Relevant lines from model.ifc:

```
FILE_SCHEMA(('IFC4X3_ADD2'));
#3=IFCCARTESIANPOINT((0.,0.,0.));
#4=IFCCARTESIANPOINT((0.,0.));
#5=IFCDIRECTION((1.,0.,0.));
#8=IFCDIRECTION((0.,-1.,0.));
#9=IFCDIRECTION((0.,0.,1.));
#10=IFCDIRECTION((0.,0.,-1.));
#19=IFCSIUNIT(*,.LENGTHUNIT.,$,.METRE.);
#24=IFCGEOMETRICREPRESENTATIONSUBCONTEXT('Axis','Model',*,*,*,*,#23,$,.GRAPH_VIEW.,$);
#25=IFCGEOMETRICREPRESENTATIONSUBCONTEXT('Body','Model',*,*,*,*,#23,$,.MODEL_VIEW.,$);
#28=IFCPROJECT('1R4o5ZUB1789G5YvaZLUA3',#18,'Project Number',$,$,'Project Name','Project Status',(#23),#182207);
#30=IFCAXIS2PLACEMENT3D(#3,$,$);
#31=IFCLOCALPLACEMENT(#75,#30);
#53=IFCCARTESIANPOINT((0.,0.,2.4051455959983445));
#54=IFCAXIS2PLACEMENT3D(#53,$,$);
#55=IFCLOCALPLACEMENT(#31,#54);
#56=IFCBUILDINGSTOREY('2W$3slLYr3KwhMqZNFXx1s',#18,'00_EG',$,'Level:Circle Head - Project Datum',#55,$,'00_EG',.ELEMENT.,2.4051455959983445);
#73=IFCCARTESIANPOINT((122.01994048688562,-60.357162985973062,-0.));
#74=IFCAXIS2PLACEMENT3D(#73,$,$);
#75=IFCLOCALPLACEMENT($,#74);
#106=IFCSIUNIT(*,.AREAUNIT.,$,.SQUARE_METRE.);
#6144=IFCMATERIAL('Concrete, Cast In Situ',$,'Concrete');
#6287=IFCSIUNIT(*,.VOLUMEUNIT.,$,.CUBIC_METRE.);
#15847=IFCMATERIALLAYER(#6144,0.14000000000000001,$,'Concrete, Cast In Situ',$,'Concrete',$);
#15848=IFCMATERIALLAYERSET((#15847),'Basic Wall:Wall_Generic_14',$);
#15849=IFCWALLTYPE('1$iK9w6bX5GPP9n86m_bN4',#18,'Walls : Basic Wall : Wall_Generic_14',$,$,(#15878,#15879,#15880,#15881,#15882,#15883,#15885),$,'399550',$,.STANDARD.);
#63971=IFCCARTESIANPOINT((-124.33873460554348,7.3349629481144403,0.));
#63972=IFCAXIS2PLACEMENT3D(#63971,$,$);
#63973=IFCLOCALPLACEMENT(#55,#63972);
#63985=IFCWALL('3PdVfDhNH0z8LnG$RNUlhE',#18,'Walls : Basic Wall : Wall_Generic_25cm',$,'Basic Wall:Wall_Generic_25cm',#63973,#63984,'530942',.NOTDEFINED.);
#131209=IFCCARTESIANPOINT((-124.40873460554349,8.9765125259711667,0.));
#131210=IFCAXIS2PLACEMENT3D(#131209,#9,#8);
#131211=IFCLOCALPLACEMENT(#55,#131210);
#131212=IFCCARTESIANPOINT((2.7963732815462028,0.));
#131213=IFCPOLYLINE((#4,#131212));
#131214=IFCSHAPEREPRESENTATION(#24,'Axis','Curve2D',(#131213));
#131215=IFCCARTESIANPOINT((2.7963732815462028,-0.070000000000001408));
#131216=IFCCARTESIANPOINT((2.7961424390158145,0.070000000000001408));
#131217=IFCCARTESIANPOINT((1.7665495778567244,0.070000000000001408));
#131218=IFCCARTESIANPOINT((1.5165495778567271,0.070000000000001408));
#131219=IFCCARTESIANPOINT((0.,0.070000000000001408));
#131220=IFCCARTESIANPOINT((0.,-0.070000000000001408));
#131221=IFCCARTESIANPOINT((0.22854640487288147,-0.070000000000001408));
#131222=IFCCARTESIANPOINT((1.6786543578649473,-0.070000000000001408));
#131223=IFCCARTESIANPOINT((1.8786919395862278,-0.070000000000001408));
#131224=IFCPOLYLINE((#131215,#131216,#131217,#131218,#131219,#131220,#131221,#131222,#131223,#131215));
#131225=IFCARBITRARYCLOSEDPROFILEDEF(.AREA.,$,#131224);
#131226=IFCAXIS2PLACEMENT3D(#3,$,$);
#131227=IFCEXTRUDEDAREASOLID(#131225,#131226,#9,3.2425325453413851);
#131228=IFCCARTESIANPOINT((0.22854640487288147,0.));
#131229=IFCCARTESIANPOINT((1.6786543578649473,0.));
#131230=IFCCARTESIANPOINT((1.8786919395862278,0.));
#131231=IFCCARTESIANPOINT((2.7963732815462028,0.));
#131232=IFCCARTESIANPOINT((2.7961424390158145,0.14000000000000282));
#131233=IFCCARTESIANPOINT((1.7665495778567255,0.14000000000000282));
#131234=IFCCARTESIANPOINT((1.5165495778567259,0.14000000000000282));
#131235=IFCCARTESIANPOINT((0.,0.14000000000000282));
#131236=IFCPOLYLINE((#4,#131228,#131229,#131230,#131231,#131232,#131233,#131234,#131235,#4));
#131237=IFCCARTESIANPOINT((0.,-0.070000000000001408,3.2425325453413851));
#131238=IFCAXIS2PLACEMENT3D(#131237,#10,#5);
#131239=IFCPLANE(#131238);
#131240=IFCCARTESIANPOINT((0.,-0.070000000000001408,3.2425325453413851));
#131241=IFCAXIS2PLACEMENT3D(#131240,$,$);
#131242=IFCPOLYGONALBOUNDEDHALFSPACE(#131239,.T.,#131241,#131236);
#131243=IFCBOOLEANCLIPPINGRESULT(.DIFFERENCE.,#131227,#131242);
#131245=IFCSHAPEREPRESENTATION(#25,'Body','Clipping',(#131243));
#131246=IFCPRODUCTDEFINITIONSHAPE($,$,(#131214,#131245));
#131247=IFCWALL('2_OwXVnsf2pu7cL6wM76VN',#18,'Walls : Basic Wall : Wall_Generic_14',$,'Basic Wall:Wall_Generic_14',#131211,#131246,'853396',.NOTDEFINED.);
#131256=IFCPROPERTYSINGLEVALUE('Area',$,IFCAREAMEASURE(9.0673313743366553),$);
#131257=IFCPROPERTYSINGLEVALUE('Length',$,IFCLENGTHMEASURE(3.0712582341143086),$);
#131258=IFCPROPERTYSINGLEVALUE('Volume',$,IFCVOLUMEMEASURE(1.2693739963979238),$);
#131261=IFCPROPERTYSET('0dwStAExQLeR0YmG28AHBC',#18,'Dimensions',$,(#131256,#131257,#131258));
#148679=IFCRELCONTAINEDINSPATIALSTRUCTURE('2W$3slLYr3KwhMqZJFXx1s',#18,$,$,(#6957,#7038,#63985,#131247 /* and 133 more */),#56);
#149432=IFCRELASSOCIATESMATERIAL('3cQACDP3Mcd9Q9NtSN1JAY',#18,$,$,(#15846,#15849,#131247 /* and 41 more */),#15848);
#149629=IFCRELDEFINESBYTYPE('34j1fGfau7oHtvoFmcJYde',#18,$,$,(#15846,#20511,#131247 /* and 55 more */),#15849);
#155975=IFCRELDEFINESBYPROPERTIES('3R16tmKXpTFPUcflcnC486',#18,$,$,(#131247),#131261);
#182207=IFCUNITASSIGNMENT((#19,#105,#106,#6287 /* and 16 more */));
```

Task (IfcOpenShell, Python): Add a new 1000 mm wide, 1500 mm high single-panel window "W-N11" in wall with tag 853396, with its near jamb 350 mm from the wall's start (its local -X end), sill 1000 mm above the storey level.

```python
import numpy as np
import ifcopenshell
import ifcopenshell.api.feature
import ifcopenshell.api.geometry
import ifcopenshell.api.pset
import ifcopenshell.api.root
import ifcopenshell.api.spatial
import ifcopenshell.geom
import ifcopenshell.util.element
import ifcopenshell.util.placement
import ifcopenshell.util.representation
import ifcopenshell.util.shape
import ifcopenshell.util.unit

model = ifcopenshell.open("model.ifc")
unit_scale = ifcopenshell.util.unit.calculate_unit_scale(model)
area_scale = ifcopenshell.util.unit.calculate_unit_scale(model, "AREAUNIT")
volume_scale = ifcopenshell.util.unit.calculate_unit_scale(model, "VOLUMEUNIT")
settings = ifcopenshell.geom.settings()


def volume(element):
    """Net volume in cubic metres, openings subtracted."""
    shape = ifcopenshell.geom.create_shape(settings, element)
    return ifcopenshell.util.shape.get_volume(shape.geometry)


wall = model.by_guid("2_OwXVnsf2pu7cL6wM76VN")
storey = ifcopenshell.util.element.get_container(wall, ifc_class="IfcBuildingStorey")
context = ifcopenshell.util.representation.get_context(model, "Model", "Body", "MODEL_VIEW")
before = volume(wall)

width, height, from_end, sill = 1, 1.5, 0.35, 1  # metres

# The wall runs along its own X axis, and the end named is its -X end.
wall_shape = ifcopenshell.geom.create_shape(settings, wall)
x, y, z = ifcopenshell.util.shape.get_vertices(wall_shape.geometry).T
start = x.min() + from_end
face, thickness = float(y.min()), float(y.max() - y.min())
wall_matrix = ifcopenshell.util.placement.get_local_placement(wall.ObjectPlacement)
level = ifcopenshell.util.placement.get_local_placement(storey.ObjectPlacement)[2, 3]


def in_wall(x, y):
    """Placement at x, y metres in the wall's axes, at sill height."""
    matrix = wall_matrix.copy()
    matrix[:, 3] = wall_matrix @ np.array([x / unit_scale, y / unit_scale, 0.0, 1.0])
    matrix[2, 3] = level + sill / unit_scale
    return matrix


# Opening: a box that overshoots both wall faces by 50 mm.
opening = ifcopenshell.api.root.create_entity(model, ifc_class="IfcOpeningElement", predefined_type="OPENING")
box = ifcopenshell.api.geometry.add_wall_representation(
    model, context=context, length=width, height=height, thickness=thickness + 0.1
)
ifcopenshell.api.geometry.assign_representation(model, product=opening, representation=box)
ifcopenshell.api.geometry.edit_object_placement(model, product=opening, matrix=in_wall(start, face - 0.05), is_si=False)
ifcopenshell.api.feature.add_feature(model, feature=opening, element=wall)

window = ifcopenshell.api.root.create_entity(model, ifc_class="IfcWindow", name="W-N11", predefined_type="WINDOW")
window.OverallWidth, window.OverallHeight = width / unit_scale, height / unit_scale
window.PartitioningType = "SINGLE_PANEL"
body = ifcopenshell.api.geometry.add_window_representation(
    model,
    context=context,
    overall_width=window.OverallWidth,
    overall_height=window.OverallHeight,
    partition_type="SINGLE_PANEL",
)
ifcopenshell.api.geometry.assign_representation(model, product=window, representation=body)
ifcopenshell.api.spatial.assign_container(model, products=[window], relating_structure=storey)
ifcopenshell.api.feature.add_filling(model, opening=opening, element=window)

# Centre the window in the wall's thickness.
ifcopenshell.api.geometry.edit_object_placement(model, product=window, matrix=in_wall(start, face), is_si=False)
window_shape = ifcopenshell.geom.create_shape(settings, window)
depth = ifcopenshell.util.shape.get_vertices(window_shape.geometry)[:, 1]
offset = face + thickness / 2 - (depth.min() + depth.max()) / 2
ifcopenshell.api.geometry.edit_object_placement(model, product=window, matrix=in_wall(start, offset), is_si=False)

after = volume(wall)

# Update the wall's stored quantities.
pset = model.by_id(ifcopenshell.util.element.get_pset(wall, "Dimensions", should_inherit=False)["id"])
ifcopenshell.api.pset.edit_pset(model, pset=pset, properties={
    "Area": model.create_entity("IfcAreaMeasure", after / thickness / area_scale),
    "Volume": model.create_entity("IfcVolumeMeasure", after / volume_scale),
})

print(f"wall volume {before:.3f} -> {after:.3f} m3")

model.write("model_v2.ifc")
```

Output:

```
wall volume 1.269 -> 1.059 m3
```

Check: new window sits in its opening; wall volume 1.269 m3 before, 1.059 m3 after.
